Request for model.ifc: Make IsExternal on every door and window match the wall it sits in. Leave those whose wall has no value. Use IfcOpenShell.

First a look at what the model holds.

```python
import ifcopenshell
import ifcopenshell.util.element

model = ifcopenshell.open("model.ifc")
print(model.schema)
seen = {}
for e in model.by_type("IfcDoor") + model.by_type("IfcWindow"):
    if not e.FillsVoids:
        continue
    host = e.FillsVoids[0].RelatingOpeningElement.VoidsElements[0].RelatingBuildingElement
    own = ifcopenshell.util.element.get_pset(e, f"Pset_{e.is_a()[3:].removesuffix('StandardCase')}Common", "IsExternal")
    wall = ifcopenshell.util.element.get_pset(host, "Pset_WallCommon", "IsExternal")
    seen[e.is_a(), own, wall] = seen.get((e.is_a(), own, wall), 0) + 1
for (cls, own, wall), count in sorted(seen.items(), key=str):
    print(count, cls, "IsExternal:", own, "| host wall:", wall)
```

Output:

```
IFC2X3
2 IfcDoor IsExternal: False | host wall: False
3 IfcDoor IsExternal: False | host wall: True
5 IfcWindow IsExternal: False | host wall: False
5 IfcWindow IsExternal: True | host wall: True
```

```python
import ifcopenshell
import ifcopenshell.api.pset
import ifcopenshell.util.element

model = ifcopenshell.open("model.ifc")

count = 0
for ifc_class, pset_name in (("IfcDoor", "Pset_DoorCommon"), ("IfcWindow", "Pset_WindowCommon")):
    for e in model.by_type(ifc_class):
        if not e.FillsVoids:
            continue
        host = e.FillsVoids[0].RelatingOpeningElement.VoidsElements[0].RelatingBuildingElement
        external = ifcopenshell.util.element.get_pset(host, "Pset_WallCommon", "IsExternal")
        if external is None or ifcopenshell.util.element.get_pset(e, pset_name, "IsExternal") == external:
            continue
        pset = ifcopenshell.api.pset.add_pset(model, product=e, name=pset_name)
        ifcopenshell.api.pset.edit_pset(model, pset=pset, properties={"IsExternal": external})
        count += 1

print(count, "updated")

model.write("model_v2.ifc")
```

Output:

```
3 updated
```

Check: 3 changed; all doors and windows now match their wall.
